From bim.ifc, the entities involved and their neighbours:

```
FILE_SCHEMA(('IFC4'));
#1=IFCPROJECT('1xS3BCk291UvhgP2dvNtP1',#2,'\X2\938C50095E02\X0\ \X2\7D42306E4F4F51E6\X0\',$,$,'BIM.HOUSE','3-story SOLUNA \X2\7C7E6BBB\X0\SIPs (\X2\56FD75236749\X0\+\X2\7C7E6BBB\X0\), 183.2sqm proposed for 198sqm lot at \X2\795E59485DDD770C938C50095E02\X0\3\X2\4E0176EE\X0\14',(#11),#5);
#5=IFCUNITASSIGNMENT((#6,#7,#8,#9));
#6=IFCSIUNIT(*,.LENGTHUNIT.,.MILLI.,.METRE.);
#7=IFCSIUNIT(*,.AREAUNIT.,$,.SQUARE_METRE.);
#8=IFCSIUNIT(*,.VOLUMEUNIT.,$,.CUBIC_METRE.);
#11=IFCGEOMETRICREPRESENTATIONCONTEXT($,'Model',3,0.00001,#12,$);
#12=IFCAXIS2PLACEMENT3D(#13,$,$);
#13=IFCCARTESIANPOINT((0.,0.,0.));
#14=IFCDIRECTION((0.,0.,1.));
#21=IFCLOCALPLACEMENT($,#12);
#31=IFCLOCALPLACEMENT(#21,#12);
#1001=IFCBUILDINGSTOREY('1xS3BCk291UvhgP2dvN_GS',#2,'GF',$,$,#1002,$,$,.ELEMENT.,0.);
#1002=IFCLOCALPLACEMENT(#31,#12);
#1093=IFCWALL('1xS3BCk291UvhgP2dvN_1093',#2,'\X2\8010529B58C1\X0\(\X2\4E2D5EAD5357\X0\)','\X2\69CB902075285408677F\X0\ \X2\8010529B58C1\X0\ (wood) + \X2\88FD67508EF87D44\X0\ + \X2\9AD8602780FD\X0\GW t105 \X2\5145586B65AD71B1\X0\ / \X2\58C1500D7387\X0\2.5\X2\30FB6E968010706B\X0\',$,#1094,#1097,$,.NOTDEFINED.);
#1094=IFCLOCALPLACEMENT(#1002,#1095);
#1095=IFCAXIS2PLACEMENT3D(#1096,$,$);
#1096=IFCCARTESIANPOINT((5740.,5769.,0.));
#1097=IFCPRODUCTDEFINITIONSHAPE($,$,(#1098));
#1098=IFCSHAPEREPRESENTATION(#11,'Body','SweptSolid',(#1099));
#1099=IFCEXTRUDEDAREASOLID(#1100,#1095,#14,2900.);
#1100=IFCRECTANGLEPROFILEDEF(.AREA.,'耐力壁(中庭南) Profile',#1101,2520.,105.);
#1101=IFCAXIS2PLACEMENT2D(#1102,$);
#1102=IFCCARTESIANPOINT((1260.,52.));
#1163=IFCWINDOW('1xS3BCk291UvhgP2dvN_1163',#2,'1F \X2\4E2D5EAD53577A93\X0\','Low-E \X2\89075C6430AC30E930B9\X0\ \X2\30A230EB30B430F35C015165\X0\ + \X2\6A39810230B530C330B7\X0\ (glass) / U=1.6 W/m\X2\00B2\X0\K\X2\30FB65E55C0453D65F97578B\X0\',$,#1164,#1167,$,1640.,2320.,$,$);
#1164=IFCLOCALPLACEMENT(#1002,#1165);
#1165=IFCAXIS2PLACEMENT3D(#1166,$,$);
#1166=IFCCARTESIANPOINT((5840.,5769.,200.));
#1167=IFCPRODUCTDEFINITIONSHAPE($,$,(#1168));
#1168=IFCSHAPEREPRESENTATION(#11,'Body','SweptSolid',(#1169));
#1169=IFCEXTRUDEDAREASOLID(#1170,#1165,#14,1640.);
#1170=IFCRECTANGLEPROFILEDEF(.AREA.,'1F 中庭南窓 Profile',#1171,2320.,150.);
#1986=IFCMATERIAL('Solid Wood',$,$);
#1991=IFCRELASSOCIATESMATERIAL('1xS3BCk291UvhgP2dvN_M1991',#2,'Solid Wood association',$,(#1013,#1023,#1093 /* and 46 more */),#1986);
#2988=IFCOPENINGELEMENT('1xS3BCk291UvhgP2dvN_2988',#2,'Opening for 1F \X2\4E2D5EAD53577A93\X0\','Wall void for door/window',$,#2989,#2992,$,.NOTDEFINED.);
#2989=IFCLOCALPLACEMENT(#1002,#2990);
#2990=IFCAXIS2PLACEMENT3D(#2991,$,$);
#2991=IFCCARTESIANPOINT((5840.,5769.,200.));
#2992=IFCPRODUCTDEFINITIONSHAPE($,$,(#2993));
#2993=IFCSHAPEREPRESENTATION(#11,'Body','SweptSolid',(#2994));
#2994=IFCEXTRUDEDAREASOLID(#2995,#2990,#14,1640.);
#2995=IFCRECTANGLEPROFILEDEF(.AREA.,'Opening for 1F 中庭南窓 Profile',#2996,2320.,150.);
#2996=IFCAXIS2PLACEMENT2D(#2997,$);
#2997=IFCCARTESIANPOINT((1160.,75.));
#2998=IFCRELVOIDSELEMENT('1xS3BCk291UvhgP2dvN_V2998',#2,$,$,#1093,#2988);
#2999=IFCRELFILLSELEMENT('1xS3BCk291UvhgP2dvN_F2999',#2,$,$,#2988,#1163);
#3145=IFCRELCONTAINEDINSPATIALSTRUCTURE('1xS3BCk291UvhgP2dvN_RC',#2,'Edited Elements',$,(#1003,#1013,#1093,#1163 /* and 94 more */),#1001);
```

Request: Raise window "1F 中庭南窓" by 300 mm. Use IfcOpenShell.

```python
import numpy as np
import ifcopenshell
import ifcopenshell.api.geometry
import ifcopenshell.util.placement
import ifcopenshell.util.unit

model = ifcopenshell.open("bim.ifc")
unit_scale = ifcopenshell.util.unit.calculate_unit_scale(model)

window = model.by_guid("1xS3BCk291UvhgP2dvN_1163")
opening = window.FillsVoids[0].RelatingOpeningElement
dz = 0.3 / unit_scale

shift = np.array([0.0, 0.0, dz])
# The window is not placed relative to its opening, so move both.
for product in (opening, window):
    matrix = ifcopenshell.util.placement.get_local_placement(product.ObjectPlacement)
    matrix[:3, 3] += shift
    ifcopenshell.api.geometry.edit_object_placement(model, product=product, matrix=matrix, is_si=False)

print(f"moved by {dz * unit_scale:+.3f} m")

model.write("bim_edited.ifc")
```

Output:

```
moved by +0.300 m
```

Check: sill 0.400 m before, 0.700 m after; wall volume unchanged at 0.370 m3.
